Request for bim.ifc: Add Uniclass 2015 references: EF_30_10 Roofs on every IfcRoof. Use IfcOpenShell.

First a look at what the model holds.

```python
import ifcopenshell

model = ifcopenshell.open("bim.ifc")
print(model.schema)
print("classifications:", [c.Name for c in model.by_type("IfcClassification")])
for ifc_class in ("IfcDoor", "IfcRoof", "IfcStair", "IfcWall", "IfcWindow"):
    print(ifc_class, len(model.by_type(ifc_class)))
```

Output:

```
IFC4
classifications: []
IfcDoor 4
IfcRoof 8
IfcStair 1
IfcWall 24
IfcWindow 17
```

```python
import ifcopenshell
import ifcopenshell.api.classification

model = ifcopenshell.open("bim.ifc")

system = ifcopenshell.api.classification.add_classification(model, classification="Uniclass 2015")

codes = {
    "IfcRoof": ("EF_30_10", "Roofs"),
}
for ifc_class, (code, name) in codes.items():
    products = model.by_type(ifc_class)
    ifcopenshell.api.classification.add_reference(
        model, products=products, classification=system, identification=code, name=name
    )
    print(code, len(products))

model.write("bim-out.ifc")
```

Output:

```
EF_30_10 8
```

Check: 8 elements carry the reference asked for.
